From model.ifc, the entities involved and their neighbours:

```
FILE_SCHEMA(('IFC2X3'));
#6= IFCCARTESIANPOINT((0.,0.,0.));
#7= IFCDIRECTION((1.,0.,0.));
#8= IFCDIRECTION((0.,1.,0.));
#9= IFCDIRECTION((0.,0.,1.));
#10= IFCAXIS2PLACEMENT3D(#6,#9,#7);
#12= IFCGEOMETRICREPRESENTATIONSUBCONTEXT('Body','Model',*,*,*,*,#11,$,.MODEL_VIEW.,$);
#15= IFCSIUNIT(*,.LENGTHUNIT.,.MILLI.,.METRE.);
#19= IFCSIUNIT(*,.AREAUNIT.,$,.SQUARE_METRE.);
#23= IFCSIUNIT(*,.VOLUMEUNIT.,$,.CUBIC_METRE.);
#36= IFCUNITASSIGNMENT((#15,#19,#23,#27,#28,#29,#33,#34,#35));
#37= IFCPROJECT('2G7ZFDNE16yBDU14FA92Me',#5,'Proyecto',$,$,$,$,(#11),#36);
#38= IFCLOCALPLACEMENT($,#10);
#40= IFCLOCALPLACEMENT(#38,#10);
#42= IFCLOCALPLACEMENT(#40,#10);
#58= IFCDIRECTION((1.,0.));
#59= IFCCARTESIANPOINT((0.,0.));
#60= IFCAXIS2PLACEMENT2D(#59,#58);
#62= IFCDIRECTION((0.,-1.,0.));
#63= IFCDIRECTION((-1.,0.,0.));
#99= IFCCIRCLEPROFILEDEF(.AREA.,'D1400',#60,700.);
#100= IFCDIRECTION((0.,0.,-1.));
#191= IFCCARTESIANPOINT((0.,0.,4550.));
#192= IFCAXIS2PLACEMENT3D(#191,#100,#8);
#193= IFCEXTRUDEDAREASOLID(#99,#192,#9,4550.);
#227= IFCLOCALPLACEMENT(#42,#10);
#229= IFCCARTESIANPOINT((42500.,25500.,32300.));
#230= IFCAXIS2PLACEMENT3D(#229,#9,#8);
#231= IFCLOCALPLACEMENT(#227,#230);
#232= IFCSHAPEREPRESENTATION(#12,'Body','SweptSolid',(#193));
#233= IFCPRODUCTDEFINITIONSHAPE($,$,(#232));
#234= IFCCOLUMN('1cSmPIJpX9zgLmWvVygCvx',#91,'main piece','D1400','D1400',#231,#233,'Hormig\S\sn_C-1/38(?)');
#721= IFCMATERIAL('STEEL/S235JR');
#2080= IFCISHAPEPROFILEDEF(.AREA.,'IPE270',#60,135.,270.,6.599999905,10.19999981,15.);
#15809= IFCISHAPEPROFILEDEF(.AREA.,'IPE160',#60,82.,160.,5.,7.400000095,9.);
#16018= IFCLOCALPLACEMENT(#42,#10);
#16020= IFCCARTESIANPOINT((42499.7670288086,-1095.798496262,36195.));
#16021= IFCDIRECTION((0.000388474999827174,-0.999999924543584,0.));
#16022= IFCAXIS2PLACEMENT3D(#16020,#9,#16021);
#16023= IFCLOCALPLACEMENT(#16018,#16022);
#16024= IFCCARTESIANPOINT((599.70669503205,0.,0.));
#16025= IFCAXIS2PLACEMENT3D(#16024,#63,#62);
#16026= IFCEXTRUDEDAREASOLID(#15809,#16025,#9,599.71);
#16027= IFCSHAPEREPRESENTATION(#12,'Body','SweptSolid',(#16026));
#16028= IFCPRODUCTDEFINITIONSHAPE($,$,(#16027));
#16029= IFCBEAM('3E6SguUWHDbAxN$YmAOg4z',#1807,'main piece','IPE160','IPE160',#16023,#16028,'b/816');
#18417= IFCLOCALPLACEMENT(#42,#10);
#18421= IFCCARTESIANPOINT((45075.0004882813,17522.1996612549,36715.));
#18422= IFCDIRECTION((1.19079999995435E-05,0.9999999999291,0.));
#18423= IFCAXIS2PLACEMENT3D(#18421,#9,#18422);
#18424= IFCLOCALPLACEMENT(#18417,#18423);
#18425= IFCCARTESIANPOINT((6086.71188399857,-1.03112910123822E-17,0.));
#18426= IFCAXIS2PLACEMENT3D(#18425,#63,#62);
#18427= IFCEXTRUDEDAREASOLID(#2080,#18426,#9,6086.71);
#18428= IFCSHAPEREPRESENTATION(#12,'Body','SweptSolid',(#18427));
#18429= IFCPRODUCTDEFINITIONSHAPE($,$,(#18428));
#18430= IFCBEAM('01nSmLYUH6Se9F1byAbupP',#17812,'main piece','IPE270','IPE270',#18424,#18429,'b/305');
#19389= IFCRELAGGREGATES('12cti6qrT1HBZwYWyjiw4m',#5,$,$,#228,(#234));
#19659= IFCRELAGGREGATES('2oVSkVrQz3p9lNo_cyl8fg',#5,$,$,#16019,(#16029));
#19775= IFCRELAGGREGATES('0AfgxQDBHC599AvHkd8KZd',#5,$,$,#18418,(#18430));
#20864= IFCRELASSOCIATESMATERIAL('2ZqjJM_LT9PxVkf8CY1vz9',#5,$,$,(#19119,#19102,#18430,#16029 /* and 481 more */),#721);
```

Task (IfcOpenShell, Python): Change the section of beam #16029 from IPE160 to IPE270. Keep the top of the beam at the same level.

```python
import ifcopenshell
import ifcopenshell.util.element
import ifcopenshell.util.representation

model = ifcopenshell.open("model.ifc")

member = model.by_guid("3E6SguUWHDbAxN$YmAOg4z")
source = next(p for p in model.by_type("IfcIShapeProfileDef") if p.ProfileName == "IPE270")

body = ifcopenshell.util.representation.get_representation(member, "Model", "Body")
solid = body.Items[0]
old_profile = solid.SweptArea

# Copy the section's sizes but keep this member's own profile position.
profile = ifcopenshell.util.element.copy(model, source)
# Profiles are centred, so shift by half the change in depth to hold the top.
shift = (old_profile.OverallDepth - profile.OverallDepth) / 2
x, y = old_profile.Position.Location.Coordinates
up = (0.0, 1.0)  # upwards, in the solid's own plane
location = model.createIfcCartesianPoint((x + up[0] * shift, y + up[1] * shift))
profile.Position = model.createIfcAxis2Placement2D(location, old_profile.Position.RefDirection)
solid.SweptArea = profile
if not model.get_total_inverses(old_profile):
    ifcopenshell.util.element.remove_deep2(model, old_profile)
member.Description = member.Description.replace("IPE160", "IPE270")
member.ObjectType = member.ObjectType.replace("IPE160", "IPE270")

print(solid.SweptArea)

model.write("model_edited.ifc")
```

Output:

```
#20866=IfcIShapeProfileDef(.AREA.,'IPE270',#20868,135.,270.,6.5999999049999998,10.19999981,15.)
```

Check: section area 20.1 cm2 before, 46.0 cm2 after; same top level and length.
